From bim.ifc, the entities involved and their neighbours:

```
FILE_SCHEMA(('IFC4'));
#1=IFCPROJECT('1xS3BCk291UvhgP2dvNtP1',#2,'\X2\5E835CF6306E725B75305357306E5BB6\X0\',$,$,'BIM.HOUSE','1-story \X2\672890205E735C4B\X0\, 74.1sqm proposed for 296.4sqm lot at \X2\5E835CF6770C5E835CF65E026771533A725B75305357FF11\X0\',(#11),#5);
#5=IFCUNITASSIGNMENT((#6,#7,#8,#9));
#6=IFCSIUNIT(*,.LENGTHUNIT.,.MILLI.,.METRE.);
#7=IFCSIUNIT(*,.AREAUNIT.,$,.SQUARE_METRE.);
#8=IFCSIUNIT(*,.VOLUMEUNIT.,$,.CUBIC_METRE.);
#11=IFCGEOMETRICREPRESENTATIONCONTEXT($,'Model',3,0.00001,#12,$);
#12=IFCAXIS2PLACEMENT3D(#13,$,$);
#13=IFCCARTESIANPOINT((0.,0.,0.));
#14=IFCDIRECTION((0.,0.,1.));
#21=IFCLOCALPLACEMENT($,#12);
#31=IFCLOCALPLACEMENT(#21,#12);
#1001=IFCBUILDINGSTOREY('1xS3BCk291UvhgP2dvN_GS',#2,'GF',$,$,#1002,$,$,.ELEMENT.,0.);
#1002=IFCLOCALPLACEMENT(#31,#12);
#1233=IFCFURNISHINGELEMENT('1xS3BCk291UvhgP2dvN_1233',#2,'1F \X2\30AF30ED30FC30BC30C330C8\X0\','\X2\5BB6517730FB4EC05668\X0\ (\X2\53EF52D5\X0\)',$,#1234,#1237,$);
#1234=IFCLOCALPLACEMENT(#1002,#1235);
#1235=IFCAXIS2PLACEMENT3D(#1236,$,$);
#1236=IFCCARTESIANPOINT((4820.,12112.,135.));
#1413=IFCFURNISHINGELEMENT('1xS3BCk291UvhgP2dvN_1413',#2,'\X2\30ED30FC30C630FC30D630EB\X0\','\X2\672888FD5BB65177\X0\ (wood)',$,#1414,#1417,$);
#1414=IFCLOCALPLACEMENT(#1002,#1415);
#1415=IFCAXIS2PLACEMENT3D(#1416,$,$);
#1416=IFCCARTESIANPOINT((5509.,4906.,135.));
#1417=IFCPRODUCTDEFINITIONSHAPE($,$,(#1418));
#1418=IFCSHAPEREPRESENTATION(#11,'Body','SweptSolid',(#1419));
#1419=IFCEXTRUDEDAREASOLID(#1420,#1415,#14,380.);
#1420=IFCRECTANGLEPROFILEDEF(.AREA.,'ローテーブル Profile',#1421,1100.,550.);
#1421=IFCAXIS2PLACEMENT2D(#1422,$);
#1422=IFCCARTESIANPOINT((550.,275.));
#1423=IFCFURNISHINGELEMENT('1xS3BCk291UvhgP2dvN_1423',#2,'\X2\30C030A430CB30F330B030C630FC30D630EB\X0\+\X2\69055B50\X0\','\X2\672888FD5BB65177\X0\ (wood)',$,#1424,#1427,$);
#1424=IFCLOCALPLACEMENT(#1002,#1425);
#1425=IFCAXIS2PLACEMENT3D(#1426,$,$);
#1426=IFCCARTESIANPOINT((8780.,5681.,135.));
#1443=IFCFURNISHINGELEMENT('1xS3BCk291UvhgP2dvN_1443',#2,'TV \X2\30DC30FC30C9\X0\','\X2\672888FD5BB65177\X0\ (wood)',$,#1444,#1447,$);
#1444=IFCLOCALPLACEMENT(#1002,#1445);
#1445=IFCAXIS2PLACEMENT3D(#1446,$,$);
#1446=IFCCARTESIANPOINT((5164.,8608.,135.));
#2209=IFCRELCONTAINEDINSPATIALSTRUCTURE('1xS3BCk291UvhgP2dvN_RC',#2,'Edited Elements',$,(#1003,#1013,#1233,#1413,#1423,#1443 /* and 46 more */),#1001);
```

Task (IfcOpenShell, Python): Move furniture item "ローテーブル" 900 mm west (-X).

```python
import ifcopenshell
import ifcopenshell.api.geometry
import ifcopenshell.util.placement
import ifcopenshell.util.unit

model = ifcopenshell.open("bim.ifc")
unit_scale = ifcopenshell.util.unit.calculate_unit_scale(model)

item = model.by_guid("1xS3BCk291UvhgP2dvN_1413")
matrix = ifcopenshell.util.placement.get_local_placement(item.ObjectPlacement)
matrix[0, 3] -= 0.9 / unit_scale
ifcopenshell.api.geometry.edit_object_placement(model, product=item, matrix=matrix, is_si=False)

print(ifcopenshell.util.placement.get_local_placement(item.ObjectPlacement).round(3) + 0.0)

model.write("bim_edited.ifc")
```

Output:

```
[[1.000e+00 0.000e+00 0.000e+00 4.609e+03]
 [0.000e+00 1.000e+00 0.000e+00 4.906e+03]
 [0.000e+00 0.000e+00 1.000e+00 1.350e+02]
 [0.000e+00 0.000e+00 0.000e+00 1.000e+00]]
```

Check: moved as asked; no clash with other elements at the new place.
